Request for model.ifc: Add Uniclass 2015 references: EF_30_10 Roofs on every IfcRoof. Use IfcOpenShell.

First a look at what the model holds.

```python
import ifcopenshell

model = ifcopenshell.open("model.ifc")
print(model.schema)
print("classifications:", [c.Name for c in model.by_type("IfcClassification")])
for ifc_class in ("IfcDoor", "IfcRoof", "IfcStair", "IfcWall", "IfcWindow"):
    print(ifc_class, len(model.by_type(ifc_class)))
```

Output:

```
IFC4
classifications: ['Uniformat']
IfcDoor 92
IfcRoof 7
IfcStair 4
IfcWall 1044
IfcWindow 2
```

```python
import ifcopenshell
import ifcopenshell.api.classification

model = ifcopenshell.open("model.ifc")

system = ifcopenshell.api.classification.add_classification(model, classification="Uniclass 2015")

codes = {
    "IfcRoof": ("EF_30_10", "Roofs"),
}
for ifc_class, (code, name) in codes.items():
    products = model.by_type(ifc_class)
    ifcopenshell.api.classification.add_reference(
        model, products=products, classification=system, identification=code, name=name
    )
    print(code, len(products))

model.write("model_updated.ifc")
```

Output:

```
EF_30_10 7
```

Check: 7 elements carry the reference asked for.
